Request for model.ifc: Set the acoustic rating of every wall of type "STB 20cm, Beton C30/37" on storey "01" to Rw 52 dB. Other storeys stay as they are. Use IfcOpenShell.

First a look at what the model holds.

```python
import ifcopenshell
import ifcopenshell.util.element

model = ifcopenshell.open("model.ifc")
print(model.schema)
storey = next(s for s in model.by_type("IfcBuildingStorey") if s.Name == "01")
walls = [e for e in ifcopenshell.util.element.get_decomposition(storey) if e.is_a("IfcWall")]
seen = {}
for e in walls:
    element_type = ifcopenshell.util.element.get_type(e)
    key = (element_type.Name if element_type != e and element_type else None, ifcopenshell.util.element.get_pset(e, "Pset_WallCommon", "AcousticRating"))
    seen[key] = seen.get(key, 0) + 1
for (name, value), count in sorted(seen.items(), key=str):
    print(count, "x", name, "|", value)
```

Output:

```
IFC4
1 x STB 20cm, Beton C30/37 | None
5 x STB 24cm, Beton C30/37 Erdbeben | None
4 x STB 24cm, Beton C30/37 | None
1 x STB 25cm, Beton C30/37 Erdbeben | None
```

```python
import ifcopenshell
import ifcopenshell.api.pset
import ifcopenshell.util.element

model = ifcopenshell.open("model.ifc")

storey = next(s for s in model.by_type("IfcBuildingStorey") if s.Name == "01")
walls = [e for e in ifcopenshell.util.element.get_decomposition(storey) if e.is_a("IfcWall")]

count = 0
for e in walls:
    element_type = ifcopenshell.util.element.get_type(e)
    if element_type in (None, e) or element_type.Name != "STB 20cm, Beton C30/37":
        continue
    # add_pset returns the element's existing set when there is one.
    pset = ifcopenshell.api.pset.add_pset(model, product=e, name="Pset_WallCommon")
    ifcopenshell.api.pset.edit_pset(model, pset=pset, properties={"AcousticRating": "Rw 52 dB"})
    count += 1

print(count, "walls updated")

model.write("model_edited.ifc")
```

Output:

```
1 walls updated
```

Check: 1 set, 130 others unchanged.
